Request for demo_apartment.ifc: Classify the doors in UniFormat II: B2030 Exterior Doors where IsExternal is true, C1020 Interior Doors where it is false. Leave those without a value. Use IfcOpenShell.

First a look at what the model holds.

```python
import ifcopenshell
import ifcopenshell.util.element

model = ifcopenshell.open("demo_apartment.ifc")
print(model.schema)
print("classifications:", [c.Name for c in model.by_type("IfcClassification")])
values = [ifcopenshell.util.element.get_pset(e, "Pset_DoorCommon", "IsExternal") for e in model.by_type("IfcDoor")]
for value in (True, False, None):
    print("IsExternal", value, values.count(value))
```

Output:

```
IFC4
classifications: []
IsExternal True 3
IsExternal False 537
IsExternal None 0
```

```python
import ifcopenshell
import ifcopenshell.api.classification
import ifcopenshell.util.element

model = ifcopenshell.open("demo_apartment.ifc")

system = ifcopenshell.api.classification.add_classification(model, classification="UniFormat II")

doors = model.by_type("IfcDoor")
external = {e: ifcopenshell.util.element.get_pset(e, "Pset_DoorCommon", "IsExternal") for e in doors}
for flag, code, name in ((True, "B2030", "Exterior Doors"), (False, "C1020", "Interior Doors")):
    products = [e for e in doors if external[e] is flag]
    ifcopenshell.api.classification.add_reference(
        model, products=products, classification=system, identification=code, name=name
    )
    print(code, len(products))

model.write("demo_apartment-out.ifc")
```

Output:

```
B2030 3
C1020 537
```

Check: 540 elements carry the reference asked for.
